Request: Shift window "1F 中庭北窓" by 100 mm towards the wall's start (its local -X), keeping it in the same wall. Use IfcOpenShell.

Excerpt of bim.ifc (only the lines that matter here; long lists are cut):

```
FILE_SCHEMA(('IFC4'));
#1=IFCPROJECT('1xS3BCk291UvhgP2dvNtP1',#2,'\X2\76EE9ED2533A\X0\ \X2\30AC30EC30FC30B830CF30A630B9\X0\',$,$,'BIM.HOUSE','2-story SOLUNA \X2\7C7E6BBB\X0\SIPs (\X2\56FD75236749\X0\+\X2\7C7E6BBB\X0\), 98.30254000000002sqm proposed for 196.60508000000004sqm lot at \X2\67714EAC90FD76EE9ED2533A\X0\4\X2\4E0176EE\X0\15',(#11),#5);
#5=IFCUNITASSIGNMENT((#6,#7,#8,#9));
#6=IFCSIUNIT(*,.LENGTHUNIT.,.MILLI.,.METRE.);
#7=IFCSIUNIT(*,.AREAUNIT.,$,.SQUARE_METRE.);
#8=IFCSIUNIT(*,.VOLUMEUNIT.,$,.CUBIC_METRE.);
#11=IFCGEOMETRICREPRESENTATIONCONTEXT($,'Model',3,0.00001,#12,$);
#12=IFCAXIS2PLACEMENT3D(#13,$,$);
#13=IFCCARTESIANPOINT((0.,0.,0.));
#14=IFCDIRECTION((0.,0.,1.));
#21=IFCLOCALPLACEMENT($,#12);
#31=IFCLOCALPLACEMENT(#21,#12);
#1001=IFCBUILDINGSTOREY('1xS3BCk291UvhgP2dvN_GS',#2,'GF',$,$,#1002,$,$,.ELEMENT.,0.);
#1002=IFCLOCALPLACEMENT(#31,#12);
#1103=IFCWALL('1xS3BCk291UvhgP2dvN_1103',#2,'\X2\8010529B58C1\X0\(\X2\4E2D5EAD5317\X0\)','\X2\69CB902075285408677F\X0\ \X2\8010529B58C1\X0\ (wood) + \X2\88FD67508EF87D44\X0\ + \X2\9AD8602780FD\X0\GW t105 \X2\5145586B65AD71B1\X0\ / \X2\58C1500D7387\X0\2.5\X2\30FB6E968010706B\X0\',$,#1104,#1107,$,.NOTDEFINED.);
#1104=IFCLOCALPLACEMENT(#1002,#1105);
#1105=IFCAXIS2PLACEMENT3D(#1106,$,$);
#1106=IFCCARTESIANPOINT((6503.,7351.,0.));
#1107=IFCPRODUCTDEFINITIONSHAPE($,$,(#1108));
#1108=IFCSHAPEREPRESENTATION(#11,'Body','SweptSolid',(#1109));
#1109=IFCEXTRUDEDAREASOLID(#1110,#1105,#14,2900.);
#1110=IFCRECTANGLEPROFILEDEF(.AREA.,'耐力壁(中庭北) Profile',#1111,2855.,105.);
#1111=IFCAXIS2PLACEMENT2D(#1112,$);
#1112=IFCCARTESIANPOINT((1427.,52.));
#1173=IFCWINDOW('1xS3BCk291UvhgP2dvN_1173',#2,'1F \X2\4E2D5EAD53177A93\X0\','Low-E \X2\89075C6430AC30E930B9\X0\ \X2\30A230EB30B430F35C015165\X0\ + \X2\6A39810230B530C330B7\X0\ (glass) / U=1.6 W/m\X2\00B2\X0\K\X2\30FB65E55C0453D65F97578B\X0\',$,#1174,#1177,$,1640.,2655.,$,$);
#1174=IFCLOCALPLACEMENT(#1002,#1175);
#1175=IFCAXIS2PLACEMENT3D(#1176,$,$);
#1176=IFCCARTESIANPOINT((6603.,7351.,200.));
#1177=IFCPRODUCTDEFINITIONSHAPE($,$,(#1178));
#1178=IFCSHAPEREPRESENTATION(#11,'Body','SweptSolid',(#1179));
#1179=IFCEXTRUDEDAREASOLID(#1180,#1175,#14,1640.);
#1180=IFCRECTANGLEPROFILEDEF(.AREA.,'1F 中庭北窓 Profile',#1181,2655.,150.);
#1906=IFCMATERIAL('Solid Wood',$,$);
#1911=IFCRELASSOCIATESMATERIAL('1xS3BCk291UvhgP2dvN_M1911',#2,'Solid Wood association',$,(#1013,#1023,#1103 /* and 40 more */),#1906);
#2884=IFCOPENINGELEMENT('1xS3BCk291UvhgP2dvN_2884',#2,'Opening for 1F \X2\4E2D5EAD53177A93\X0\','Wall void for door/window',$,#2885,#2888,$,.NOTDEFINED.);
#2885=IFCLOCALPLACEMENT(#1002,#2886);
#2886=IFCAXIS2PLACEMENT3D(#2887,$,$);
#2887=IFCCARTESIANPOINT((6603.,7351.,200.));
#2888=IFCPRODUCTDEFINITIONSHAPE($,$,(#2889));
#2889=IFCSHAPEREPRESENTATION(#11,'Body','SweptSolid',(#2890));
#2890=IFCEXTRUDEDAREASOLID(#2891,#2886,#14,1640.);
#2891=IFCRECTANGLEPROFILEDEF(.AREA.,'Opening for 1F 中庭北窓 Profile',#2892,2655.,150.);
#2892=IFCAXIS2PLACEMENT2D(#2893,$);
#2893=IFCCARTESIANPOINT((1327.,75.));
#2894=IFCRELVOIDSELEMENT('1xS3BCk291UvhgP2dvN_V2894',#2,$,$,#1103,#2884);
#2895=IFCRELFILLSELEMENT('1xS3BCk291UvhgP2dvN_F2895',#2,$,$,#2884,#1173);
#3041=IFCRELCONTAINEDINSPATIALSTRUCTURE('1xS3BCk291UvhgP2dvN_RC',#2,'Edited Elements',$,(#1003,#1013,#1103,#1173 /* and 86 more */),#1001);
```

```python
import ifcopenshell
import ifcopenshell.api.geometry
import ifcopenshell.util.placement

model = ifcopenshell.open("bim.ifc")

window = model.by_guid("1xS3BCk291UvhgP2dvN_1173")
opening = window.FillsVoids[0].RelatingOpeningElement
wall = opening.VoidsElements[0].RelatingBuildingElement

wall_matrix = ifcopenshell.util.placement.get_local_placement(wall.ObjectPlacement)
shift = wall_matrix[:3, 0] * -100.0
before = ifcopenshell.util.placement.get_local_placement(window.ObjectPlacement)[:3, 3].copy()

# The window is not placed relative to its opening, so move both.
for product in (opening, window):
    matrix = ifcopenshell.util.placement.get_local_placement(product.ObjectPlacement)
    matrix[:3, 3] += shift
    ifcopenshell.api.geometry.edit_object_placement(model, product=product, matrix=matrix, is_si=False)

after = ifcopenshell.util.placement.get_local_placement(window.ObjectPlacement)[:3, 3]
print("window moved by", (after - before).round(3) + 0.0)

model.write("bim_v2.ifc")
```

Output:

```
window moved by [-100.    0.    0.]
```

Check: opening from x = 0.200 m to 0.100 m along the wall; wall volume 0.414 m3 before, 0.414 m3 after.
